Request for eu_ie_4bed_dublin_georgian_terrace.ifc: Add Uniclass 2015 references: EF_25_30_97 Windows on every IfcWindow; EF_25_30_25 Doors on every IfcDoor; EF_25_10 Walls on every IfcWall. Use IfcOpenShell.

First a look at what the model holds.

```python
import ifcopenshell

model = ifcopenshell.open("eu_ie_4bed_dublin_georgian_terrace.ifc")
print(model.schema)
print("classifications:", [c.Name for c in model.by_type("IfcClassification")])
for ifc_class in ("IfcDoor", "IfcRoof", "IfcStair", "IfcWall", "IfcWindow"):
    print(ifc_class, len(model.by_type(ifc_class)))
```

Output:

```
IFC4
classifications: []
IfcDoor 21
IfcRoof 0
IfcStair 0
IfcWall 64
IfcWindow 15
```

```python
import ifcopenshell
import ifcopenshell.api.classification

model = ifcopenshell.open("eu_ie_4bed_dublin_georgian_terrace.ifc")

system = ifcopenshell.api.classification.add_classification(model, classification="Uniclass 2015")

codes = {
    "IfcWindow": ("EF_25_30_97", "Windows"),
    "IfcDoor": ("EF_25_30_25", "Doors"),
    "IfcWall": ("EF_25_10", "Walls"),
}
for ifc_class, (code, name) in codes.items():
    products = model.by_type(ifc_class)
    ifcopenshell.api.classification.add_reference(
        model, products=products, classification=system, identification=code, name=name
    )
    print(code, len(products))

model.write("eu_ie_4bed_dublin_georgian_terrace_rev.ifc")
```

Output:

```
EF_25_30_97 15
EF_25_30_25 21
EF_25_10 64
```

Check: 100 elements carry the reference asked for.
